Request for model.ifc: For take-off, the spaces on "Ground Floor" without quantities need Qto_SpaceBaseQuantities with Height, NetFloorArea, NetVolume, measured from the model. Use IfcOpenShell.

First a look at what the model holds.

```python
import ifcopenshell
import ifcopenshell.util.element
import ifcopenshell.util.unit

model = ifcopenshell.open("model.ifc")
print(model.schema)
for unit_type in ("LENGTHUNIT", "AREAUNIT", "VOLUMEUNIT"):
    print(unit_type, ifcopenshell.util.unit.calculate_unit_scale(model, unit_type))
storey = next(s for s in model.by_type("IfcBuildingStorey") if s.Name == "Ground Floor")
spaces = [e for e in ifcopenshell.util.element.get_decomposition(storey) if e.is_a("IfcSpace")]
for e in sorted(spaces, key=lambda e: e.id()):
    print(e.id(), e.is_a(), e.Name, list(ifcopenshell.util.element.get_psets(e, qtos_only=True)), sep=" | ")
```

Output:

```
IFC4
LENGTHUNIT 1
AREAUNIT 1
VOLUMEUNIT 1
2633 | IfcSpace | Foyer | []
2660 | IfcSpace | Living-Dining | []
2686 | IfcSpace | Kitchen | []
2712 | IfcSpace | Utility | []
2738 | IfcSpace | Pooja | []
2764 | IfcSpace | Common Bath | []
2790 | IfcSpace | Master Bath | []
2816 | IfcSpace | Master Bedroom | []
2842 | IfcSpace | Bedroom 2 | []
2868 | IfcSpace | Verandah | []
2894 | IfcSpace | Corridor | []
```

```python
import ifcopenshell
import ifcopenshell.api.pset
import ifcopenshell.geom
import ifcopenshell.util.element
import ifcopenshell.util.shape
import ifcopenshell.util.unit

model = ifcopenshell.open("model.ifc")
unit_scale = ifcopenshell.util.unit.calculate_unit_scale(model)
area_scale = ifcopenshell.util.unit.calculate_unit_scale(model, "AREAUNIT")
volume_scale = ifcopenshell.util.unit.calculate_unit_scale(model, "VOLUMEUNIT")
settings = ifcopenshell.geom.settings()

storey = next(s for s in model.by_type("IfcBuildingStorey") if s.Name == "Ground Floor")
spaces = [e for e in ifcopenshell.util.element.get_decomposition(storey) if e.is_a("IfcSpace")]

for e in sorted(spaces, key=lambda e: e.id()):
    if ifcopenshell.util.element.get_psets(e, qtos_only=True, should_inherit=False):
        continue
    # Geometry comes back in metres, in the element's own axes.
    shape = ifcopenshell.geom.create_shape(settings, e)
    values = {
        "Height": ifcopenshell.util.shape.get_z(shape.geometry) / unit_scale,
        "NetFloorArea": ifcopenshell.util.shape.get_footprint_area(shape.geometry) / area_scale,
        "NetVolume": ifcopenshell.util.shape.get_volume(shape.geometry) / volume_scale,
    }
    qto = ifcopenshell.api.pset.add_qto(model, product=e, name="Qto_SpaceBaseQuantities")
    ifcopenshell.api.pset.edit_qto(model, qto=qto, properties=values)
    print(e.id(), {k: round(v, 3) for k, v in values.items()})

model.write("model_rev.ifc")
```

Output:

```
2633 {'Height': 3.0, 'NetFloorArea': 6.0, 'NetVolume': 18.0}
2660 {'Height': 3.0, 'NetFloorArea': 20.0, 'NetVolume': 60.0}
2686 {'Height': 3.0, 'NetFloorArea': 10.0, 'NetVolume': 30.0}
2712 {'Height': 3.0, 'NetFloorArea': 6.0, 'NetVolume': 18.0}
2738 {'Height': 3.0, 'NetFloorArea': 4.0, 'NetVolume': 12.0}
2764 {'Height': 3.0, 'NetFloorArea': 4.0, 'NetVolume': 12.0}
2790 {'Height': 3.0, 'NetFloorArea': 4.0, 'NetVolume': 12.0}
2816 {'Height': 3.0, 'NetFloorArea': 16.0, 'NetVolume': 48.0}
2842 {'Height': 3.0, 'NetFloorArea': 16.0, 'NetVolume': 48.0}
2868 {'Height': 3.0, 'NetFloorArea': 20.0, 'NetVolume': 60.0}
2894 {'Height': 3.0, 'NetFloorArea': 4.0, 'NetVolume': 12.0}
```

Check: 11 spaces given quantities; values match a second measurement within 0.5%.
